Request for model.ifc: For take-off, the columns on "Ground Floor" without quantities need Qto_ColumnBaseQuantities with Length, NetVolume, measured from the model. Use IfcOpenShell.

First a look at what the model holds.

```python
import ifcopenshell
import ifcopenshell.util.element
import ifcopenshell.util.unit

model = ifcopenshell.open("model.ifc")
print(model.schema)
for unit_type in ("LENGTHUNIT", "AREAUNIT", "VOLUMEUNIT"):
    print(unit_type, ifcopenshell.util.unit.calculate_unit_scale(model, unit_type))
storey = next(s for s in model.by_type("IfcBuildingStorey") if s.Name == "Ground Floor")
columns = [e for e in ifcopenshell.util.element.get_decomposition(storey) if e.is_a("IfcColumn")]
for e in sorted(columns, key=lambda e: e.id()):
    print(e.id(), e.is_a(), e.Name, list(ifcopenshell.util.element.get_psets(e, qtos_only=True)), sep=" | ")
```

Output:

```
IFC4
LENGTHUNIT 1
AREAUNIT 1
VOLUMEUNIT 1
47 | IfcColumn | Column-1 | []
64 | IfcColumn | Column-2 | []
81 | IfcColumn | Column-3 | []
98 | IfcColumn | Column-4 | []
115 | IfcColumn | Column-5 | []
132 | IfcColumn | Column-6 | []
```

```python
import ifcopenshell
import ifcopenshell.api.pset
import ifcopenshell.geom
import ifcopenshell.util.element
import ifcopenshell.util.shape
import ifcopenshell.util.unit

model = ifcopenshell.open("model.ifc")
unit_scale = ifcopenshell.util.unit.calculate_unit_scale(model)
volume_scale = ifcopenshell.util.unit.calculate_unit_scale(model, "VOLUMEUNIT")
settings = ifcopenshell.geom.settings()

storey = next(s for s in model.by_type("IfcBuildingStorey") if s.Name == "Ground Floor")
columns = [e for e in ifcopenshell.util.element.get_decomposition(storey) if e.is_a("IfcColumn")]

for e in sorted(columns, key=lambda e: e.id()):
    if ifcopenshell.util.element.get_psets(e, qtos_only=True, should_inherit=False):
        continue
    # Geometry comes back in metres, in the element's own axes.
    shape = ifcopenshell.geom.create_shape(settings, e)
    values = {
        "Length": ifcopenshell.util.shape.get_z(shape.geometry) / unit_scale,
        "NetVolume": ifcopenshell.util.shape.get_volume(shape.geometry) / volume_scale,
    }
    qto = ifcopenshell.api.pset.add_qto(model, product=e, name="Qto_ColumnBaseQuantities")
    ifcopenshell.api.pset.edit_qto(model, qto=qto, properties=values)
    print(e.id(), {k: round(v, 3) for k, v in values.items()})

model.write("model-out.ifc")
```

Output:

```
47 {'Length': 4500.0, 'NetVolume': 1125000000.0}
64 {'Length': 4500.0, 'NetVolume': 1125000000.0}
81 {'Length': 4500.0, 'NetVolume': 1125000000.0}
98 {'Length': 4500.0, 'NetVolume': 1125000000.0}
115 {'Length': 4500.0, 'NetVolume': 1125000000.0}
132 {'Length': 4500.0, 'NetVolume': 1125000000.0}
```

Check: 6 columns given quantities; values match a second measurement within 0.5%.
